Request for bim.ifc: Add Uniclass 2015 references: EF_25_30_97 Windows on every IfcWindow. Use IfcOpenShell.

First a look at what the model holds.

```python
import ifcopenshell

model = ifcopenshell.open("bim.ifc")
print(model.schema)
print("classifications:", [c.Name for c in model.by_type("IfcClassification")])
for ifc_class in ("IfcDoor", "IfcRoof", "IfcStair", "IfcWall", "IfcWindow"):
    print(ifc_class, len(model.by_type(ifc_class)))
```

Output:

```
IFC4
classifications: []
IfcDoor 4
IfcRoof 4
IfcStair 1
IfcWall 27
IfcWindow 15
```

```python
import ifcopenshell
import ifcopenshell.api.classification

model = ifcopenshell.open("bim.ifc")

system = ifcopenshell.api.classification.add_classification(model, classification="Uniclass 2015")

codes = {
    "IfcWindow": ("EF_25_30_97", "Windows"),
}
for ifc_class, (code, name) in codes.items():
    products = model.by_type(ifc_class)
    ifcopenshell.api.classification.add_reference(
        model, products=products, classification=system, identification=code, name=name
    )
    print(code, len(products))

model.write("bim_updated.ifc")
```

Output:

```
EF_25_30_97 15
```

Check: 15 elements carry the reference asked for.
